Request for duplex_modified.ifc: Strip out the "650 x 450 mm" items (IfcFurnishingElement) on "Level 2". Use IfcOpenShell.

First a look at what the model holds.

```python
import ifcopenshell
import ifcopenshell.util.element

model = ifcopenshell.open("duplex_modified.ifc")
print(model.schema)
storey = next(s for s in model.by_type("IfcBuildingStorey") if s.Name == "Level 2")
furniture = [e for e in ifcopenshell.util.element.get_decomposition(storey) if e.is_a("IfcFurnishingElement")]
seen = {}
for e in furniture:
    element_type = ifcopenshell.util.element.get_type(e)
    name = element_type.Name if element_type not in (None, e) else None
    seen[name] = seen.get(name, 0) + 1
for name, count in sorted(seen.items(), key=str):
    print(count, "x", name)
```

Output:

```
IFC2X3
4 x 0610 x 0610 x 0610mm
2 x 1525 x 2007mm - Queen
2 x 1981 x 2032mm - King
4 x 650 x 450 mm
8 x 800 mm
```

```python
import ifcopenshell
import ifcopenshell.api.root
import ifcopenshell.util.element

model = ifcopenshell.open("duplex_modified.ifc")

storey = next(s for s in model.by_type("IfcBuildingStorey") if s.Name == "Level 2")
furniture = [e for e in ifcopenshell.util.element.get_decomposition(storey) if e.is_a("IfcFurnishingElement")]
targets = [e for e in furniture if (t := ifcopenshell.util.element.get_type(e)) not in (None, e) and t.Name == "650 x 450 mm"]

for e in targets:
    ifcopenshell.api.root.remove_product(model, product=e)
print(len(targets), "removed")

model.write("duplex_modified-out.ifc")
```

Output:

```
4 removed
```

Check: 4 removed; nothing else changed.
